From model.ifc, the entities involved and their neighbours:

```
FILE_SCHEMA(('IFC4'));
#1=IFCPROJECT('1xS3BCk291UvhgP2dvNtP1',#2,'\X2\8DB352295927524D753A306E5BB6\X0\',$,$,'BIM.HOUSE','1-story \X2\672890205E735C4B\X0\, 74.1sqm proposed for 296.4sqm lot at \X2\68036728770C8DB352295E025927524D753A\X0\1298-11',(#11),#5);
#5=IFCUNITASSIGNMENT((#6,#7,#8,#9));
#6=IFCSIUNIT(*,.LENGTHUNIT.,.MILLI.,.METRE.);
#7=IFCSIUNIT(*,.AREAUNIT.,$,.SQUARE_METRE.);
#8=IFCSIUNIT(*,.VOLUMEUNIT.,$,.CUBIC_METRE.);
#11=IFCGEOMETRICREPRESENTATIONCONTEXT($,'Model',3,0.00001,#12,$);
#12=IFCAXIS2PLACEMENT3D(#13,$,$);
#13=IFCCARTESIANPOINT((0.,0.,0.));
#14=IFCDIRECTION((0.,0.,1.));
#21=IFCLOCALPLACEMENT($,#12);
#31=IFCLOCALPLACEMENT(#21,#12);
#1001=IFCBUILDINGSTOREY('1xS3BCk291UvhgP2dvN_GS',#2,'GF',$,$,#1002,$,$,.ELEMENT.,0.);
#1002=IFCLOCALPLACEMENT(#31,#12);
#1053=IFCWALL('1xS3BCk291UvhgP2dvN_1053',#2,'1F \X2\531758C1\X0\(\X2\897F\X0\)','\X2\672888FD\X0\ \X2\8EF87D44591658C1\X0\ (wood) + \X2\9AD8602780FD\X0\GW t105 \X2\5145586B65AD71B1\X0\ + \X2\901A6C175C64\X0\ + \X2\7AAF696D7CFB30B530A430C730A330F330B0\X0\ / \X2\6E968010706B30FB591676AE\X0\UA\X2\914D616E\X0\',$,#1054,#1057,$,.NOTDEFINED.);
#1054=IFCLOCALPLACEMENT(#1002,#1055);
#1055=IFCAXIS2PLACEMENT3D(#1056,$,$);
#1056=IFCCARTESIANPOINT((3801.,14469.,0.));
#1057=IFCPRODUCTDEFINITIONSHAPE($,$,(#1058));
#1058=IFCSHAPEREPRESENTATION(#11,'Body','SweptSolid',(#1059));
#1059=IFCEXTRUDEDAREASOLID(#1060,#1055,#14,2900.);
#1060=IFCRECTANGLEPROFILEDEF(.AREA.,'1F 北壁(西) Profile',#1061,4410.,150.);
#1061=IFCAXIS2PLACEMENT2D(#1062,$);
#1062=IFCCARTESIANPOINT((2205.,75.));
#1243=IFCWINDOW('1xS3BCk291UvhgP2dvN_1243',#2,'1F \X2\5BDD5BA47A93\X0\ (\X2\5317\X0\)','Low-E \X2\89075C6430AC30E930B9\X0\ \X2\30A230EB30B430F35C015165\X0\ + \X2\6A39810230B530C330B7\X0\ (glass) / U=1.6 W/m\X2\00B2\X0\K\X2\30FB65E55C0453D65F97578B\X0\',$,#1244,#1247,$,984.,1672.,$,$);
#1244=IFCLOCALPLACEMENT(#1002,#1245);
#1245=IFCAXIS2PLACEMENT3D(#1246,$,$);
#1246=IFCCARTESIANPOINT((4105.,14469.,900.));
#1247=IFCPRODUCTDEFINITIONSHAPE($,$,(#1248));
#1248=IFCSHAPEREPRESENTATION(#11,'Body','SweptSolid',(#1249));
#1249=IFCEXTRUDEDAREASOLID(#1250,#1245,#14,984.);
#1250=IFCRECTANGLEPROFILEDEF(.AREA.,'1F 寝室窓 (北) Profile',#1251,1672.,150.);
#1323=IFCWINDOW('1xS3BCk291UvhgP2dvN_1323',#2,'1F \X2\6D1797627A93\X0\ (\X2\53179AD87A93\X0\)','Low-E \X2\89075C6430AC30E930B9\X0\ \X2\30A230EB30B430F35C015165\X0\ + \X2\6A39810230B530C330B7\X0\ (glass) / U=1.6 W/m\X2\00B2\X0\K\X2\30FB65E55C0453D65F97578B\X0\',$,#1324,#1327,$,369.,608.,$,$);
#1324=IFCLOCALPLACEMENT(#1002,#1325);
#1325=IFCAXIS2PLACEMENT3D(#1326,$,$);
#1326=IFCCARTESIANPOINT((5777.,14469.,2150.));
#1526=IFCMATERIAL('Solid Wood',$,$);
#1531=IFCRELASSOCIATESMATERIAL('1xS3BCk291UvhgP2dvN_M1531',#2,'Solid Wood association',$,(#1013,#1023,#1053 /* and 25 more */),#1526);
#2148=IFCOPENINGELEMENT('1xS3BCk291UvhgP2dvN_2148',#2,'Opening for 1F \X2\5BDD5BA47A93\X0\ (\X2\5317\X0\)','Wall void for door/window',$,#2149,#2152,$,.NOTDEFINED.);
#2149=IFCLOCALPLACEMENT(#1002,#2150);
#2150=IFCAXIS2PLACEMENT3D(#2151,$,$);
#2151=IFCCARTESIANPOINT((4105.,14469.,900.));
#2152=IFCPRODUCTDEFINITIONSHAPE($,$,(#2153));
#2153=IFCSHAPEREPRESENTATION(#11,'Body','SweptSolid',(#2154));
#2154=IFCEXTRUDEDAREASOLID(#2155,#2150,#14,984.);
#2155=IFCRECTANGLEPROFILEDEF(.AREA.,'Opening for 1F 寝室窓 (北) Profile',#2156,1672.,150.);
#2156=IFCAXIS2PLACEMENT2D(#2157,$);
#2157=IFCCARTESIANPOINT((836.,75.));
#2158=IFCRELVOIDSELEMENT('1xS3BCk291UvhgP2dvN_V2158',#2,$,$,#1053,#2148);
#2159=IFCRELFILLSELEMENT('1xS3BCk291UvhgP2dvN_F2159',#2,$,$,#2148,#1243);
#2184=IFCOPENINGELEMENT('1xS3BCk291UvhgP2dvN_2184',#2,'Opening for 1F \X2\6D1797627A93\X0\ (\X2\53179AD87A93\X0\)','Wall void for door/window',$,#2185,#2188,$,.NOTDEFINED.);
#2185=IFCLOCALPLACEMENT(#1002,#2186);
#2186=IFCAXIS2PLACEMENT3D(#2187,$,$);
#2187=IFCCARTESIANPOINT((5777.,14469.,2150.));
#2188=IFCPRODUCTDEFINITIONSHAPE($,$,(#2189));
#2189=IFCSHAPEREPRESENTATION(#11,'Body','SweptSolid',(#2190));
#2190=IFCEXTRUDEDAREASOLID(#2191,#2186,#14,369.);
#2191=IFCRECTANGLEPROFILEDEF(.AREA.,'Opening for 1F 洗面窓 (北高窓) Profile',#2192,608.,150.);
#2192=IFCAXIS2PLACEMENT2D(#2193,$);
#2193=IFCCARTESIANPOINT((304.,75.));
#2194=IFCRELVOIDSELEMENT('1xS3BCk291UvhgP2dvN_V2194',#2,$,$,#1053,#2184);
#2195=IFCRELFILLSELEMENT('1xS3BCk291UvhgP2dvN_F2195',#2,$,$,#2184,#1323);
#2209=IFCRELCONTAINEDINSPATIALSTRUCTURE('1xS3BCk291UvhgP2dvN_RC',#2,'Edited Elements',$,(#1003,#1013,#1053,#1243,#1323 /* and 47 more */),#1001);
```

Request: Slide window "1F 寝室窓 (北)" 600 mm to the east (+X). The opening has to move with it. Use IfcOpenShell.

```python
import ifcopenshell
import ifcopenshell.api.geometry
import ifcopenshell.util.placement

model = ifcopenshell.open("model.ifc")

window = model.by_guid("1xS3BCk291UvhgP2dvN_1243")
opening = window.FillsVoids[0].RelatingOpeningElement
wall = opening.VoidsElements[0].RelatingBuildingElement

wall_matrix = ifcopenshell.util.placement.get_local_placement(wall.ObjectPlacement)
shift = wall_matrix[:3, 0] * 600.0
before = ifcopenshell.util.placement.get_local_placement(window.ObjectPlacement)[:3, 3].copy()

# The window is not placed relative to its opening, so move both.
for product in (opening, window):
    matrix = ifcopenshell.util.placement.get_local_placement(product.ObjectPlacement)
    matrix[:3, 3] += shift
    ifcopenshell.api.geometry.edit_object_placement(model, product=product, matrix=matrix, is_si=False)

after = ifcopenshell.util.placement.get_local_placement(window.ObjectPlacement)[:3, 3]
print("window moved by", (after - before).round(3) + 0.0)

model.write("model_rev.ifc")
```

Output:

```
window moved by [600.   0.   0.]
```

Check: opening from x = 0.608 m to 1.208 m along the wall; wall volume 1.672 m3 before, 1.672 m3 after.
